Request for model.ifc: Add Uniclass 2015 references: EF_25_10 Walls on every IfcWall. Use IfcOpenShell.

First a look at what the model holds.

```python
import ifcopenshell

model = ifcopenshell.open("model.ifc")
print(model.schema)
print("classifications:", [c.Name for c in model.by_type("IfcClassification")])
for ifc_class in ("IfcDoor", "IfcRoof", "IfcStair", "IfcWall", "IfcWindow"):
    print(ifc_class, len(model.by_type(ifc_class)))
```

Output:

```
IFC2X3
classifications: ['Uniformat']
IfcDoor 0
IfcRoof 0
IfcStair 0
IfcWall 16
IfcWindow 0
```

```python
import ifcopenshell
import ifcopenshell.api.classification

model = ifcopenshell.open("model.ifc")

# IFC2X3 requires Source and Edition and has no link from the project to the system.
system = model.create_entity("IfcClassification", Source="NBS", Edition="2015", Name="Uniclass 2015")

codes = {
    "IfcWall": ("EF_25_10", "Walls"),
}
for ifc_class, (code, name) in codes.items():
    products = model.by_type(ifc_class)
    ifcopenshell.api.classification.add_reference(
        model, products=products, classification=system, identification=code, name=name
    )
    print(code, len(products))

model.write("model-out.ifc")
```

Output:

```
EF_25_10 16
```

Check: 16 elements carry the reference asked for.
